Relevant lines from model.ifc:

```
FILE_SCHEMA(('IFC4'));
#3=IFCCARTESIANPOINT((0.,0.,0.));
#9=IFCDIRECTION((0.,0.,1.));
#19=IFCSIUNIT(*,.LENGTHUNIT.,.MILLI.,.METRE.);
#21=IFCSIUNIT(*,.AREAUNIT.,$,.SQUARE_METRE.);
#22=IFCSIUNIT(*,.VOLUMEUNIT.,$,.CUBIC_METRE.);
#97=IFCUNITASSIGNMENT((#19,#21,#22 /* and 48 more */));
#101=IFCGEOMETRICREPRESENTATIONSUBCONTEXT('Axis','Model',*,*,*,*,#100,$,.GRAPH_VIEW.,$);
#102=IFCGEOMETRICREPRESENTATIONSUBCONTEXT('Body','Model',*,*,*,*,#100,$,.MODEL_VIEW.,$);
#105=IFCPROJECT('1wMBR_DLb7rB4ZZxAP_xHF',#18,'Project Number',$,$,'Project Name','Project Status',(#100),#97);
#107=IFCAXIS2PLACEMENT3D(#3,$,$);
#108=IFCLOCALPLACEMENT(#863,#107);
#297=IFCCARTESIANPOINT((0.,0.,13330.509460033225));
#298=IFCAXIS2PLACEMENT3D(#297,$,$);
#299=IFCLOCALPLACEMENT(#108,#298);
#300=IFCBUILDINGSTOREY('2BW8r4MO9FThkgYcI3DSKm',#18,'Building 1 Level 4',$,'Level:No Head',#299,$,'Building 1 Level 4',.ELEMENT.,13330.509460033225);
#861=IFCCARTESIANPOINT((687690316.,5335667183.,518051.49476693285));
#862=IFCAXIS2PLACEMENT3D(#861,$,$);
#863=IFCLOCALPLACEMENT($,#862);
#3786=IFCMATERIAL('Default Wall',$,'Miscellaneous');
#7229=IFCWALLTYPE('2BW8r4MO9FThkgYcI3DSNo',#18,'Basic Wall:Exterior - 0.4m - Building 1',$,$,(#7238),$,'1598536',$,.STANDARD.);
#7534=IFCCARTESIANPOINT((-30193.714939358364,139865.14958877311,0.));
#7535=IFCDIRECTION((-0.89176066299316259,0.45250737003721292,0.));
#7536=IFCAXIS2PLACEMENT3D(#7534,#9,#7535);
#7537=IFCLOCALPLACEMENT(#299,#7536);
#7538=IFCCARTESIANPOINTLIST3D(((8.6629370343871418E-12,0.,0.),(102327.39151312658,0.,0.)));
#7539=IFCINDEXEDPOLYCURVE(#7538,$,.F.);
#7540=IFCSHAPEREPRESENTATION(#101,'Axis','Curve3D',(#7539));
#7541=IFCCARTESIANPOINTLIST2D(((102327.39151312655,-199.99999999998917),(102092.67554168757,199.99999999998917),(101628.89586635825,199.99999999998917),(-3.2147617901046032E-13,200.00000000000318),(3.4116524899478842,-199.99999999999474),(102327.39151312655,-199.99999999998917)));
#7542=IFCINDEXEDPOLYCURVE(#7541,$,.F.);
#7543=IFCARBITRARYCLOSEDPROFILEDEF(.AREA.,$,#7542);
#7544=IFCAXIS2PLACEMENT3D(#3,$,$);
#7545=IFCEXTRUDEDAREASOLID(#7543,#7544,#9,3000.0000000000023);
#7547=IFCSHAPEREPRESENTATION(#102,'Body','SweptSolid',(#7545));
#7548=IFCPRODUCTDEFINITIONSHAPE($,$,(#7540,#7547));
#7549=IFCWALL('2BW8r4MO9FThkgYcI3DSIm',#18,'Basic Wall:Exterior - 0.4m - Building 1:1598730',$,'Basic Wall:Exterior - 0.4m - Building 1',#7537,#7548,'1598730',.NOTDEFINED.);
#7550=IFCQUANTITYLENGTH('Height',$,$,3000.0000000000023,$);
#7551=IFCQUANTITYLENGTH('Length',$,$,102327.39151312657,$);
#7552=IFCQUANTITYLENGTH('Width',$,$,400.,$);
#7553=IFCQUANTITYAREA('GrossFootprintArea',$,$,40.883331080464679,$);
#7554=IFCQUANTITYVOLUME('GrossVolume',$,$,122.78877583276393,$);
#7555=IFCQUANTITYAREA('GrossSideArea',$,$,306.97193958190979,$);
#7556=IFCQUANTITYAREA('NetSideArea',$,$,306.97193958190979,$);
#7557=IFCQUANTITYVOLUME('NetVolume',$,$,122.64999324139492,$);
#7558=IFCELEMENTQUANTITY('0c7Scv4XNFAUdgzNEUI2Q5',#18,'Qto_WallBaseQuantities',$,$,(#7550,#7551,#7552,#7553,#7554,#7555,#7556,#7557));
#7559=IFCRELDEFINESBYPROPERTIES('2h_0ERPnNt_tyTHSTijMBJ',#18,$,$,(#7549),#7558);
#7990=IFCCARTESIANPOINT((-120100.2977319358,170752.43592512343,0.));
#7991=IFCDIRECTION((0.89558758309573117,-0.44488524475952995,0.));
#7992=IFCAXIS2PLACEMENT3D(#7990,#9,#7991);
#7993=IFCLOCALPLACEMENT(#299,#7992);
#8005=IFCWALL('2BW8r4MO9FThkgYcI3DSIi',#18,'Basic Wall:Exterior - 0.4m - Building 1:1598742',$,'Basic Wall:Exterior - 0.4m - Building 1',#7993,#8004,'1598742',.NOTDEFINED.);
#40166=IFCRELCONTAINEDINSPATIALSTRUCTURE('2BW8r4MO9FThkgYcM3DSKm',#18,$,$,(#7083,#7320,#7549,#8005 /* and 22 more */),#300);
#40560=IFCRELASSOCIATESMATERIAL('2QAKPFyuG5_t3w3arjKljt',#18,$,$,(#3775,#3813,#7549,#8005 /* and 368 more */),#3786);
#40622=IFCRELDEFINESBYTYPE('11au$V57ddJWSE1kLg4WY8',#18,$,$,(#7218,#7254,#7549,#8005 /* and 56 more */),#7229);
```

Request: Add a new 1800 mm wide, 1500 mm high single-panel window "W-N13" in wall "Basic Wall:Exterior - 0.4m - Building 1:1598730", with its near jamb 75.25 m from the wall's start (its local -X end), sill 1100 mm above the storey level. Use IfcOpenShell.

```python
import numpy as np
import ifcopenshell
import ifcopenshell.api.feature
import ifcopenshell.api.geometry
import ifcopenshell.api.pset
import ifcopenshell.api.root
import ifcopenshell.api.spatial
import ifcopenshell.geom
import ifcopenshell.util.element
import ifcopenshell.util.placement
import ifcopenshell.util.representation
import ifcopenshell.util.shape
import ifcopenshell.util.unit

model = ifcopenshell.open("model.ifc")
unit_scale = ifcopenshell.util.unit.calculate_unit_scale(model)
area_scale = ifcopenshell.util.unit.calculate_unit_scale(model, "AREAUNIT")
volume_scale = ifcopenshell.util.unit.calculate_unit_scale(model, "VOLUMEUNIT")
settings = ifcopenshell.geom.settings()


def volume(element):
    """Net volume in cubic metres, openings subtracted."""
    shape = ifcopenshell.geom.create_shape(settings, element)
    return ifcopenshell.util.shape.get_volume(shape.geometry)


wall = model.by_id(7549)
storey = ifcopenshell.util.element.get_container(wall, ifc_class="IfcBuildingStorey")
context = ifcopenshell.util.representation.get_context(model, "Model", "Body", "MODEL_VIEW")
before = volume(wall)

width, height, from_end, sill = 1.8, 1.5, 75.25, 1.1  # metres

# The wall runs along its own X axis, and the end named is its -X end.
wall_shape = ifcopenshell.geom.create_shape(settings, wall)
x, y, z = ifcopenshell.util.shape.get_vertices(wall_shape.geometry).T
start = x.min() + from_end
face, thickness = float(y.min()), float(y.max() - y.min())
wall_matrix = ifcopenshell.util.placement.get_local_placement(wall.ObjectPlacement)
level = ifcopenshell.util.placement.get_local_placement(storey.ObjectPlacement)[2, 3]


def in_wall(x, y):
    """Placement at x, y metres in the wall's axes, at sill height."""
    matrix = wall_matrix.copy()
    matrix[:, 3] = wall_matrix @ np.array([x / unit_scale, y / unit_scale, 0.0, 1.0])
    matrix[2, 3] = level + sill / unit_scale
    return matrix


# Opening: a box that overshoots both wall faces by 50 mm.
opening = ifcopenshell.api.root.create_entity(model, ifc_class="IfcOpeningElement", predefined_type="OPENING")
box = ifcopenshell.api.geometry.add_wall_representation(
    model, context=context, length=width, height=height, thickness=thickness + 0.1
)
ifcopenshell.api.geometry.assign_representation(model, product=opening, representation=box)
ifcopenshell.api.geometry.edit_object_placement(model, product=opening, matrix=in_wall(start, face - 0.05), is_si=False)
ifcopenshell.api.feature.add_feature(model, feature=opening, element=wall)

window = ifcopenshell.api.root.create_entity(model, ifc_class="IfcWindow", name="W-N13", predefined_type="WINDOW")
window.OverallWidth, window.OverallHeight = width / unit_scale, height / unit_scale
window.PartitioningType = "SINGLE_PANEL"
body = ifcopenshell.api.geometry.add_window_representation(
    model,
    context=context,
    overall_width=window.OverallWidth,
    overall_height=window.OverallHeight,
    partition_type="SINGLE_PANEL",
)
ifcopenshell.api.geometry.assign_representation(model, product=window, representation=body)
ifcopenshell.api.spatial.assign_container(model, products=[window], relating_structure=storey)
ifcopenshell.api.feature.add_filling(model, opening=opening, element=window)

# Centre the window in the wall's thickness.
ifcopenshell.api.geometry.edit_object_placement(model, product=window, matrix=in_wall(start, face), is_si=False)
window_shape = ifcopenshell.geom.create_shape(settings, window)
depth = ifcopenshell.util.shape.get_vertices(window_shape.geometry)[:, 1]
offset = face + thickness / 2 - (depth.min() + depth.max()) / 2
ifcopenshell.api.geometry.edit_object_placement(model, product=window, matrix=in_wall(start, offset), is_si=False)

after = volume(wall)

# Update the wall's stored quantities.
qto = model.by_id(ifcopenshell.util.element.get_pset(wall, "Qto_WallBaseQuantities", should_inherit=False)["id"])
ifcopenshell.api.pset.edit_qto(model, qto=qto, properties={
    "NetSideArea": after / thickness / area_scale,
    "NetVolume": after / volume_scale,
})

print(f"wall volume {before:.3f} -> {after:.3f} m3")

model.write("model_updated.ifc")
```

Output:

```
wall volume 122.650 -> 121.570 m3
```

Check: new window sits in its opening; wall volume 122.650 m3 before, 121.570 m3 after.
